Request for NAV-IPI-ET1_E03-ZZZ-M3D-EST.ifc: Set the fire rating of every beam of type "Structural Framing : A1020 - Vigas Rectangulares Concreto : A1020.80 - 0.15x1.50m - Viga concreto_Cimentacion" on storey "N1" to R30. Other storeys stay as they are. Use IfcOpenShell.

First a look at what the model holds.

```python
import ifcopenshell
import ifcopenshell.util.element

model = ifcopenshell.open("NAV-IPI-ET1_E03-ZZZ-M3D-EST.ifc")
print(model.schema)
storey = next(s for s in model.by_type("IfcBuildingStorey") if s.Name == "N1")
beams = [e for e in ifcopenshell.util.element.get_decomposition(storey) if e.is_a("IfcBeam")]
seen = {}
for e in beams:
    element_type = ifcopenshell.util.element.get_type(e)
    key = (element_type.Name if element_type != e and element_type else None, ifcopenshell.util.element.get_pset(e, "Pset_BeamCommon", "FireRating"))
    seen[key] = seen.get(key, 0) + 1
for (name, value), count in sorted(seen.items(), key=str):
    print(count, "x", name, "|", value)
```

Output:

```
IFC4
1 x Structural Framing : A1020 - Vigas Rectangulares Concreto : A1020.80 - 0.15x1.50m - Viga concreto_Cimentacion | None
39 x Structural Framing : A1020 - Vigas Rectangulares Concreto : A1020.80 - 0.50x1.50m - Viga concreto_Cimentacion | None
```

```python
import ifcopenshell
import ifcopenshell.api.pset
import ifcopenshell.util.element

model = ifcopenshell.open("NAV-IPI-ET1_E03-ZZZ-M3D-EST.ifc")

storey = next(s for s in model.by_type("IfcBuildingStorey") if s.Name == "N1")
beams = [e for e in ifcopenshell.util.element.get_decomposition(storey) if e.is_a("IfcBeam")]

count = 0
for e in beams:
    element_type = ifcopenshell.util.element.get_type(e)
    if element_type in (None, e) or element_type.Name != "Structural Framing : A1020 - Vigas Rectangulares Concreto : A1020.80 - 0.15x1.50m - Viga concreto_Cimentacion":
        continue
    # add_pset returns the element's existing set when there is one.
    pset = ifcopenshell.api.pset.add_pset(model, product=e, name="Pset_BeamCommon")
    ifcopenshell.api.pset.edit_pset(model, pset=pset, properties={"FireRating": "R30"})
    count += 1

print(count, "beams updated")

model.write("NAV-IPI-ET1_E03-ZZZ-M3D-EST_updated.ifc")
```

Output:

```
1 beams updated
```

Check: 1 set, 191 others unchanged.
